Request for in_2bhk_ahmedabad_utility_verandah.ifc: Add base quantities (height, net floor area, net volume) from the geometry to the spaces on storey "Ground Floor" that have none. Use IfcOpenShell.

First a look at what the model holds.

```python
import ifcopenshell
import ifcopenshell.util.element
import ifcopenshell.util.unit

model = ifcopenshell.open("in_2bhk_ahmedabad_utility_verandah.ifc")
print(model.schema)
for unit_type in ("LENGTHUNIT", "AREAUNIT", "VOLUMEUNIT"):
    print(unit_type, ifcopenshell.util.unit.calculate_unit_scale(model, unit_type))
storey = next(s for s in model.by_type("IfcBuildingStorey") if s.Name == "Ground Floor")
spaces = [e for e in ifcopenshell.util.element.get_decomposition(storey) if e.is_a("IfcSpace")]
for e in sorted(spaces, key=lambda e: e.id()):
    print(e.id(), e.is_a(), e.Name, list(ifcopenshell.util.element.get_psets(e, qtos_only=True)), sep=" | ")
```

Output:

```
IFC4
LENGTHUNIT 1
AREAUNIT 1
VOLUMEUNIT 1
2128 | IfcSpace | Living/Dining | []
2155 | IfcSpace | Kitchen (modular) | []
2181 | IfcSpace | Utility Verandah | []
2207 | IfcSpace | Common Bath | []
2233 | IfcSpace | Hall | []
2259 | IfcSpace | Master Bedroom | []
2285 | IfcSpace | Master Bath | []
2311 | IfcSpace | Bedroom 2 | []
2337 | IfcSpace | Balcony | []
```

```python
import ifcopenshell
import ifcopenshell.api.pset
import ifcopenshell.geom
import ifcopenshell.util.element
import ifcopenshell.util.shape
import ifcopenshell.util.unit

model = ifcopenshell.open("in_2bhk_ahmedabad_utility_verandah.ifc")
unit_scale = ifcopenshell.util.unit.calculate_unit_scale(model)
area_scale = ifcopenshell.util.unit.calculate_unit_scale(model, "AREAUNIT")
volume_scale = ifcopenshell.util.unit.calculate_unit_scale(model, "VOLUMEUNIT")
settings = ifcopenshell.geom.settings()

storey = next(s for s in model.by_type("IfcBuildingStorey") if s.Name == "Ground Floor")
spaces = [e for e in ifcopenshell.util.element.get_decomposition(storey) if e.is_a("IfcSpace")]

for e in sorted(spaces, key=lambda e: e.id()):
    if ifcopenshell.util.element.get_psets(e, qtos_only=True, should_inherit=False):
        continue
    # Geometry comes back in metres, in the element's own axes.
    shape = ifcopenshell.geom.create_shape(settings, e)
    values = {
        "Height": ifcopenshell.util.shape.get_z(shape.geometry) / unit_scale,
        "NetFloorArea": ifcopenshell.util.shape.get_footprint_area(shape.geometry) / area_scale,
        "NetVolume": ifcopenshell.util.shape.get_volume(shape.geometry) / volume_scale,
    }
    qto = ifcopenshell.api.pset.add_qto(model, product=e, name="Qto_SpaceBaseQuantities")
    ifcopenshell.api.pset.edit_qto(model, qto=qto, properties=values)
    print(e.id(), {k: round(v, 3) for k, v in values.items()})

model.write("in_2bhk_ahmedabad_utility_verandah_rev.ifc")
```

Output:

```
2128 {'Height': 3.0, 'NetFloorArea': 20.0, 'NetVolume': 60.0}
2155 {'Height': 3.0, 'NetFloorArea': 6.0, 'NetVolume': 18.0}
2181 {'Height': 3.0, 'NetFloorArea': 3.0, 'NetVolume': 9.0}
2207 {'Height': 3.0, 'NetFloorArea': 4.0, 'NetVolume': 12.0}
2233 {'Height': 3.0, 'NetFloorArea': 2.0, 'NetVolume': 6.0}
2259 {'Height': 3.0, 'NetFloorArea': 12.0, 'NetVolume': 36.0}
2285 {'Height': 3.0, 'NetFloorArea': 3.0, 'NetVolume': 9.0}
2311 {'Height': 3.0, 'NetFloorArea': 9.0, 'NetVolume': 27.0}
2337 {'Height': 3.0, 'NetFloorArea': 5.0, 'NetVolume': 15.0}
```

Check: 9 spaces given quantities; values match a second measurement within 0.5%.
